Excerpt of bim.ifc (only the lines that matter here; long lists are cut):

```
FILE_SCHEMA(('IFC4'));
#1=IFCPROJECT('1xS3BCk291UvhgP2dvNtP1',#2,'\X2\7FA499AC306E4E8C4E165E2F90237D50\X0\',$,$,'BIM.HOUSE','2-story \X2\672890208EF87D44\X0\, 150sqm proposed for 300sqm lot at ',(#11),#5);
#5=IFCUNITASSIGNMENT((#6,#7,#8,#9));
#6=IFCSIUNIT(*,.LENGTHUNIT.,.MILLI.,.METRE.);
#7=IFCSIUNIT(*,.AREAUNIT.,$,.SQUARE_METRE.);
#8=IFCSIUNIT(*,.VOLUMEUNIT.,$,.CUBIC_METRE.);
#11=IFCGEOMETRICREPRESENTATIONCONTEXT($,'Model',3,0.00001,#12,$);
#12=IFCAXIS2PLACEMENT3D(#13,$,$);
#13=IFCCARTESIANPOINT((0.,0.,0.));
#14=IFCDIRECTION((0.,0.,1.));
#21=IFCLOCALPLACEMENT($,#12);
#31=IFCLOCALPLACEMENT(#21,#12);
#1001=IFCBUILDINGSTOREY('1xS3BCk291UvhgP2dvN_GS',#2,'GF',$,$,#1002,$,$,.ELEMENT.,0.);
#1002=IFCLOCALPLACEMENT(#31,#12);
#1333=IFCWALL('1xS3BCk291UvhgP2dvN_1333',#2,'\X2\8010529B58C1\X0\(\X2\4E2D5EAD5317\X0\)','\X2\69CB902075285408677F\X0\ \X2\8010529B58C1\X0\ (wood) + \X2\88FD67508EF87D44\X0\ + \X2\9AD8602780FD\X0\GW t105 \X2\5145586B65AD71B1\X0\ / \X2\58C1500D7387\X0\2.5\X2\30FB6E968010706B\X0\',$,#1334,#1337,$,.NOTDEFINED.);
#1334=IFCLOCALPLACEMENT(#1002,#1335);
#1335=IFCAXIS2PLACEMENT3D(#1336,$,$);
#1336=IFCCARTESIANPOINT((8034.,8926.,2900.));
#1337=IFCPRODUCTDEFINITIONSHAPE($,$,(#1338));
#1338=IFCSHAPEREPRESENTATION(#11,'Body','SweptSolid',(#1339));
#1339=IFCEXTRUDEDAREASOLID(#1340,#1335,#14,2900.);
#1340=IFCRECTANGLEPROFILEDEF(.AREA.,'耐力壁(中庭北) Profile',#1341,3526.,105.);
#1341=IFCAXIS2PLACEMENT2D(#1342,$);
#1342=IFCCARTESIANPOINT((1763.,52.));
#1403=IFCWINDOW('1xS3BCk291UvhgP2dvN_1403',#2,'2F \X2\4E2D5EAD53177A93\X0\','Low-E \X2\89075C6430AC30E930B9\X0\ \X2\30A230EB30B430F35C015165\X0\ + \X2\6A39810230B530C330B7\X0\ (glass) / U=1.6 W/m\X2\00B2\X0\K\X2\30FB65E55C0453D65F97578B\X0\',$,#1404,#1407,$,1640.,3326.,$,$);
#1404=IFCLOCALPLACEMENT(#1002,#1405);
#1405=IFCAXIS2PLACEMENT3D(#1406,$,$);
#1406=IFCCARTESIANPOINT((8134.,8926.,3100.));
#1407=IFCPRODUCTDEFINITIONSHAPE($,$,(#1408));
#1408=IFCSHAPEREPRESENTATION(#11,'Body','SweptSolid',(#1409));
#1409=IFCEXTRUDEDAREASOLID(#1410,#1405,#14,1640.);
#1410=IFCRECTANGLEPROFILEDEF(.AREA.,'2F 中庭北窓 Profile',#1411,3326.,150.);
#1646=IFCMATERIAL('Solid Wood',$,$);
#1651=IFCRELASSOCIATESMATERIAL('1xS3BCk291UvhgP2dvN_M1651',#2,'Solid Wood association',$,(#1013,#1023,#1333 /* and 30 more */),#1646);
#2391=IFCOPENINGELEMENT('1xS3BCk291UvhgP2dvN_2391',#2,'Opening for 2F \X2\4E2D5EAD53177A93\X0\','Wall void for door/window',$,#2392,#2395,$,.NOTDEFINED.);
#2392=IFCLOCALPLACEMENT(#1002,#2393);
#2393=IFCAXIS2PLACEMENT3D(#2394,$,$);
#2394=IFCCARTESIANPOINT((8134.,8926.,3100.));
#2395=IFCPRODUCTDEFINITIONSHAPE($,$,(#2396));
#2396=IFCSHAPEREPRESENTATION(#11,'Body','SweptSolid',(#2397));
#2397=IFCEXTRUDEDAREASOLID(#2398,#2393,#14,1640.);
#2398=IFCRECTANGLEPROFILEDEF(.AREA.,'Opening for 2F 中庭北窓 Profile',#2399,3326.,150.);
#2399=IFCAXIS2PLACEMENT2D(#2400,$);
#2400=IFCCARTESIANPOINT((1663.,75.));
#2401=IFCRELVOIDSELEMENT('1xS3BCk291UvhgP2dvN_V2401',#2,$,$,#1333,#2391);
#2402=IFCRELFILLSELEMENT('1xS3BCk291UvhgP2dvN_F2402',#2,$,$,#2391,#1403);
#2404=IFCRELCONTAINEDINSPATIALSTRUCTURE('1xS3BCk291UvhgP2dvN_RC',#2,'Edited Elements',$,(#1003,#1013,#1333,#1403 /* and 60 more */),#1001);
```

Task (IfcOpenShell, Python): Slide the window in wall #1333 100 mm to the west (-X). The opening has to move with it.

```python
import ifcopenshell
import ifcopenshell.api.geometry
import ifcopenshell.util.placement

model = ifcopenshell.open("bim.ifc")

window = model.by_guid("1xS3BCk291UvhgP2dvN_1403")
opening = window.FillsVoids[0].RelatingOpeningElement
wall = opening.VoidsElements[0].RelatingBuildingElement

wall_matrix = ifcopenshell.util.placement.get_local_placement(wall.ObjectPlacement)
shift = wall_matrix[:3, 0] * -100.0
before = ifcopenshell.util.placement.get_local_placement(window.ObjectPlacement)[:3, 3].copy()

# The window is not placed relative to its opening, so move both.
for product in (opening, window):
    matrix = ifcopenshell.util.placement.get_local_placement(product.ObjectPlacement)
    matrix[:3, 3] += shift
    ifcopenshell.api.geometry.edit_object_placement(model, product=product, matrix=matrix, is_si=False)

after = ifcopenshell.util.placement.get_local_placement(window.ObjectPlacement)[:3, 3]
print("window moved by", (after - before).round(3) + 0.0)

model.write("bim_v2.ifc")
```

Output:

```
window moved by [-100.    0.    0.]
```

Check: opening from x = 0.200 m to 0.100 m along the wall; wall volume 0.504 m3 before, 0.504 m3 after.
